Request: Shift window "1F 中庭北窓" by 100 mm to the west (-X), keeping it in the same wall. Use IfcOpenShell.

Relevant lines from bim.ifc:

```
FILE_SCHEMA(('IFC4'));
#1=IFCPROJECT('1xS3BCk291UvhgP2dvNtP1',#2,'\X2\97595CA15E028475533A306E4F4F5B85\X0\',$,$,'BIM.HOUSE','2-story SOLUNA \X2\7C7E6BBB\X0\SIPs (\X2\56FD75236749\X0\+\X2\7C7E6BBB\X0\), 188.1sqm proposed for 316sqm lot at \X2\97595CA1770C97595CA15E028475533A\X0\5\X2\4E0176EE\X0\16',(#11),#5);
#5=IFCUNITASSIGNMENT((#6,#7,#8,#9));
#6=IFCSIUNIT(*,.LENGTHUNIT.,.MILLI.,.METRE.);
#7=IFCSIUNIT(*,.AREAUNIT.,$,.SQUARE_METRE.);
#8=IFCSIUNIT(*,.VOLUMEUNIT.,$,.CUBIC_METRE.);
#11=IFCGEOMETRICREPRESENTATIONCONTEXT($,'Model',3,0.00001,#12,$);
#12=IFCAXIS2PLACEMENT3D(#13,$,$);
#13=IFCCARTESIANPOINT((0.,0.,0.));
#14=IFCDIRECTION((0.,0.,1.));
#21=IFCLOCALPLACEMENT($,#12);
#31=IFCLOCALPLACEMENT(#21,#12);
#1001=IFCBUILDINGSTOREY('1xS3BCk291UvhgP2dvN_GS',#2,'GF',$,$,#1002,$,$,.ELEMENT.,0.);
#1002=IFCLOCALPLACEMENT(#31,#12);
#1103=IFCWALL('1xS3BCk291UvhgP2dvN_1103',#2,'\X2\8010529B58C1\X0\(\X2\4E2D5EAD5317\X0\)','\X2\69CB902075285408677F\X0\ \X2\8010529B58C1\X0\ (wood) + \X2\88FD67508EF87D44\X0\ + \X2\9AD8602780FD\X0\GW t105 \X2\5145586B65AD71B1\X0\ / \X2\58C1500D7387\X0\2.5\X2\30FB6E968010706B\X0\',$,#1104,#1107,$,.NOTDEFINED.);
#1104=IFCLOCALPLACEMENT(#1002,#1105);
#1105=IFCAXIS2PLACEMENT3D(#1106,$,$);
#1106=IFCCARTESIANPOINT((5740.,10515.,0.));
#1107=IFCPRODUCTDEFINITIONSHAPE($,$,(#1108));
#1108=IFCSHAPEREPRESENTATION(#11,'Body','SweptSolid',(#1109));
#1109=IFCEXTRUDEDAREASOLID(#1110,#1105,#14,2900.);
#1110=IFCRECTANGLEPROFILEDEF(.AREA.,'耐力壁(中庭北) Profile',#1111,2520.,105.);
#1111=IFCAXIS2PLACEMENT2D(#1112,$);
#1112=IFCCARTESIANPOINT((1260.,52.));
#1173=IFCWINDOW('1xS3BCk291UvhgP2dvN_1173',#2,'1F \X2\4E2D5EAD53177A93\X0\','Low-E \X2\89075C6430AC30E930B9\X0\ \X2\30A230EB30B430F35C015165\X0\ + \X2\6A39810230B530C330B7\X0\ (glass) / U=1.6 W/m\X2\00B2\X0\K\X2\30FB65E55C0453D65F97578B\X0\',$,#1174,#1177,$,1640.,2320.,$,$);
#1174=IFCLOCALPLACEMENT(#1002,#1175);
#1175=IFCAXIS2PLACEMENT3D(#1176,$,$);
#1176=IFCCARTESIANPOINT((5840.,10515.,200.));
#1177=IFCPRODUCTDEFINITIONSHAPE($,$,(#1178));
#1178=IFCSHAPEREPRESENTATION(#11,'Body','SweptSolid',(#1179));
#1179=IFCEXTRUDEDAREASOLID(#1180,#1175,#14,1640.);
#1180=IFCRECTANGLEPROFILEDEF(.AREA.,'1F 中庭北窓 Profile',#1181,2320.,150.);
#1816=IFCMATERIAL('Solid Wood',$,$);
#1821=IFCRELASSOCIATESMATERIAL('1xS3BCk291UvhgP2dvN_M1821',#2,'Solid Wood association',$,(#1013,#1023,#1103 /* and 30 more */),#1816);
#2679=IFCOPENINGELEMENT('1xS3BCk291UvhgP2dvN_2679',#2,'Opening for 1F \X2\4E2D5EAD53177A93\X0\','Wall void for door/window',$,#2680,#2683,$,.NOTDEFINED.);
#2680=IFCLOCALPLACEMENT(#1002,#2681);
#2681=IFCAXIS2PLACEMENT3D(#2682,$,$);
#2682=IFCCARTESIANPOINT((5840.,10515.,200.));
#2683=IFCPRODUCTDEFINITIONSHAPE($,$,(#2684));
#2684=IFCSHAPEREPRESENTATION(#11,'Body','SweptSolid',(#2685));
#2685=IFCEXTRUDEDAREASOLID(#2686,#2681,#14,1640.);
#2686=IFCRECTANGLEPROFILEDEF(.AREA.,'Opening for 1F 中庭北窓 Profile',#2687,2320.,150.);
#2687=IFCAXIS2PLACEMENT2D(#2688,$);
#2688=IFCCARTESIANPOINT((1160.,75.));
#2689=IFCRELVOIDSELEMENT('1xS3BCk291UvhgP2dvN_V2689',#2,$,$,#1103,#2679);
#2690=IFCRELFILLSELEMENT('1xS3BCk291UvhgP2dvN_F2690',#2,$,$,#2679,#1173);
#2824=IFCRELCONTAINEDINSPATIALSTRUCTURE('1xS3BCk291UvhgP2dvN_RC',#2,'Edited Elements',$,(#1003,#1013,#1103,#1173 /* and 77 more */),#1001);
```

```python
import ifcopenshell
import ifcopenshell.api.geometry
import ifcopenshell.util.placement

model = ifcopenshell.open("bim.ifc")

window = model.by_guid("1xS3BCk291UvhgP2dvN_1173")
opening = window.FillsVoids[0].RelatingOpeningElement
wall = opening.VoidsElements[0].RelatingBuildingElement

wall_matrix = ifcopenshell.util.placement.get_local_placement(wall.ObjectPlacement)
shift = wall_matrix[:3, 0] * -100.0
before = ifcopenshell.util.placement.get_local_placement(window.ObjectPlacement)[:3, 3].copy()

# The window is not placed relative to its opening, so move both.
for product in (opening, window):
    matrix = ifcopenshell.util.placement.get_local_placement(product.ObjectPlacement)
    matrix[:3, 3] += shift
    ifcopenshell.api.geometry.edit_object_placement(model, product=product, matrix=matrix, is_si=False)

after = ifcopenshell.util.placement.get_local_placement(window.ObjectPlacement)[:3, 3]
print("window moved by", (after - before).round(3) + 0.0)

model.write("bim-out.ifc")
```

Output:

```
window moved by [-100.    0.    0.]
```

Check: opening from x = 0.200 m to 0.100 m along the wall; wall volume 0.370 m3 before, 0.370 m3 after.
